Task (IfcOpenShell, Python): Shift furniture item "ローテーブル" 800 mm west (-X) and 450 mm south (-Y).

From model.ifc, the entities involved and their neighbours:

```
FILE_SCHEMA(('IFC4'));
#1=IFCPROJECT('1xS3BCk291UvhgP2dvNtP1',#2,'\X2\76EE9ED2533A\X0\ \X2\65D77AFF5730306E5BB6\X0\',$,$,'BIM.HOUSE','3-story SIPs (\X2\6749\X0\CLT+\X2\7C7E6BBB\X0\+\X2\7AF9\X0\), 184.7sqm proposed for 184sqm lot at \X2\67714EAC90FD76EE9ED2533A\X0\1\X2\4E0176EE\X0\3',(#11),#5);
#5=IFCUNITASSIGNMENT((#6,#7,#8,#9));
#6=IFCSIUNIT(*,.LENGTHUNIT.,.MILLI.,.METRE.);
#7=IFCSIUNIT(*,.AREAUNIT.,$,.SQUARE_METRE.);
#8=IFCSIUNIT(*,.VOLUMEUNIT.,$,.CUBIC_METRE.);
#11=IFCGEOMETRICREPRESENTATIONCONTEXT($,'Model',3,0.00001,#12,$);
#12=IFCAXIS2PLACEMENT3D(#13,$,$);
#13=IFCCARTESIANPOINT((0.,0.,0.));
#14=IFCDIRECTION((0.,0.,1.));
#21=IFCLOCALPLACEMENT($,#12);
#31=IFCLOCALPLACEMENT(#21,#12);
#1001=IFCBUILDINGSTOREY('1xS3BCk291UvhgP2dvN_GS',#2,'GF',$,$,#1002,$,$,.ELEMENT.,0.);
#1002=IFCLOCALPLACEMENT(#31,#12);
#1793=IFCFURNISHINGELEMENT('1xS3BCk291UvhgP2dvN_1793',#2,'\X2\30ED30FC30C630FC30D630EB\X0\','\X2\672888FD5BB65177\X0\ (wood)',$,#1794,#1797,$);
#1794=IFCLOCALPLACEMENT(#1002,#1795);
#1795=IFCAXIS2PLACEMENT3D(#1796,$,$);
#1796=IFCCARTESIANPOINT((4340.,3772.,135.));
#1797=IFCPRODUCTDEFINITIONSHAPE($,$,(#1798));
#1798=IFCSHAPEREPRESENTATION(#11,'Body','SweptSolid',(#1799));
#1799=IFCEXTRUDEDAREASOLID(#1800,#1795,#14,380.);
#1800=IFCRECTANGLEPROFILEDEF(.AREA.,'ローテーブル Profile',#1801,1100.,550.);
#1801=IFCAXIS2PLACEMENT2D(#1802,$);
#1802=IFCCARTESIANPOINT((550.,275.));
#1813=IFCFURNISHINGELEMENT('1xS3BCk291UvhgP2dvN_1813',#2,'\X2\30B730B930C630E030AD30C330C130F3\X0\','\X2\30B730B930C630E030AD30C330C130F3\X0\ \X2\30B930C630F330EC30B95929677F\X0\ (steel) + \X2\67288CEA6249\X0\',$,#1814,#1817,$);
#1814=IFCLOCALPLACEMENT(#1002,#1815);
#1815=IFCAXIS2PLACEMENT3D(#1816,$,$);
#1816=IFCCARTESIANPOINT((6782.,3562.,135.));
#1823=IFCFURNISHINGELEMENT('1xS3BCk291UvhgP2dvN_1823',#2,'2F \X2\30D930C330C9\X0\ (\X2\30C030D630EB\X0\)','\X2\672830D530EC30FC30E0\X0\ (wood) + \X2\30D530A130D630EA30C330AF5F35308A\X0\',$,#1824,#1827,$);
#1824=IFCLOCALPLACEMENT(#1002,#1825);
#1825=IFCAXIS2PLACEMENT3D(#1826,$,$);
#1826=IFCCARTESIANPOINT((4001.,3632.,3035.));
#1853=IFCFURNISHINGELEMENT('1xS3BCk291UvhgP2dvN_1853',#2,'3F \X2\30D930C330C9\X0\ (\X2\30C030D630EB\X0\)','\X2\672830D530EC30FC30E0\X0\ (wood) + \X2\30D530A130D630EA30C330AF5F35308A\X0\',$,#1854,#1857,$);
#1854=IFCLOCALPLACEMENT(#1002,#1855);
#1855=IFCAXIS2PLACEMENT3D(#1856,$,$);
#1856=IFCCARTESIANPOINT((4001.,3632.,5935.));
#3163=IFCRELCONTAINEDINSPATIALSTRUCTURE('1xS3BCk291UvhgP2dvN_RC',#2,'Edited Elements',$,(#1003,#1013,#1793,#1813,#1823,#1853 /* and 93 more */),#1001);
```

```python
import ifcopenshell
import ifcopenshell.api.geometry
import ifcopenshell.util.placement
import ifcopenshell.util.unit

model = ifcopenshell.open("model.ifc")
unit_scale = ifcopenshell.util.unit.calculate_unit_scale(model)

item = model.by_id(1793)
matrix = ifcopenshell.util.placement.get_local_placement(item.ObjectPlacement)
matrix[0, 3] -= 0.8 / unit_scale
matrix[1, 3] -= 0.45 / unit_scale
ifcopenshell.api.geometry.edit_object_placement(model, product=item, matrix=matrix, is_si=False)

print(ifcopenshell.util.placement.get_local_placement(item.ObjectPlacement).round(3) + 0.0)

model.write("model-out.ifc")
```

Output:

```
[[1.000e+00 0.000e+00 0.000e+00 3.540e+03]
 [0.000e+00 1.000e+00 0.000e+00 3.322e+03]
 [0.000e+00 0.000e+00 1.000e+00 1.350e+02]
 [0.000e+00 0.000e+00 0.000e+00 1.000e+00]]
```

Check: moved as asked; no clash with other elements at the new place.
